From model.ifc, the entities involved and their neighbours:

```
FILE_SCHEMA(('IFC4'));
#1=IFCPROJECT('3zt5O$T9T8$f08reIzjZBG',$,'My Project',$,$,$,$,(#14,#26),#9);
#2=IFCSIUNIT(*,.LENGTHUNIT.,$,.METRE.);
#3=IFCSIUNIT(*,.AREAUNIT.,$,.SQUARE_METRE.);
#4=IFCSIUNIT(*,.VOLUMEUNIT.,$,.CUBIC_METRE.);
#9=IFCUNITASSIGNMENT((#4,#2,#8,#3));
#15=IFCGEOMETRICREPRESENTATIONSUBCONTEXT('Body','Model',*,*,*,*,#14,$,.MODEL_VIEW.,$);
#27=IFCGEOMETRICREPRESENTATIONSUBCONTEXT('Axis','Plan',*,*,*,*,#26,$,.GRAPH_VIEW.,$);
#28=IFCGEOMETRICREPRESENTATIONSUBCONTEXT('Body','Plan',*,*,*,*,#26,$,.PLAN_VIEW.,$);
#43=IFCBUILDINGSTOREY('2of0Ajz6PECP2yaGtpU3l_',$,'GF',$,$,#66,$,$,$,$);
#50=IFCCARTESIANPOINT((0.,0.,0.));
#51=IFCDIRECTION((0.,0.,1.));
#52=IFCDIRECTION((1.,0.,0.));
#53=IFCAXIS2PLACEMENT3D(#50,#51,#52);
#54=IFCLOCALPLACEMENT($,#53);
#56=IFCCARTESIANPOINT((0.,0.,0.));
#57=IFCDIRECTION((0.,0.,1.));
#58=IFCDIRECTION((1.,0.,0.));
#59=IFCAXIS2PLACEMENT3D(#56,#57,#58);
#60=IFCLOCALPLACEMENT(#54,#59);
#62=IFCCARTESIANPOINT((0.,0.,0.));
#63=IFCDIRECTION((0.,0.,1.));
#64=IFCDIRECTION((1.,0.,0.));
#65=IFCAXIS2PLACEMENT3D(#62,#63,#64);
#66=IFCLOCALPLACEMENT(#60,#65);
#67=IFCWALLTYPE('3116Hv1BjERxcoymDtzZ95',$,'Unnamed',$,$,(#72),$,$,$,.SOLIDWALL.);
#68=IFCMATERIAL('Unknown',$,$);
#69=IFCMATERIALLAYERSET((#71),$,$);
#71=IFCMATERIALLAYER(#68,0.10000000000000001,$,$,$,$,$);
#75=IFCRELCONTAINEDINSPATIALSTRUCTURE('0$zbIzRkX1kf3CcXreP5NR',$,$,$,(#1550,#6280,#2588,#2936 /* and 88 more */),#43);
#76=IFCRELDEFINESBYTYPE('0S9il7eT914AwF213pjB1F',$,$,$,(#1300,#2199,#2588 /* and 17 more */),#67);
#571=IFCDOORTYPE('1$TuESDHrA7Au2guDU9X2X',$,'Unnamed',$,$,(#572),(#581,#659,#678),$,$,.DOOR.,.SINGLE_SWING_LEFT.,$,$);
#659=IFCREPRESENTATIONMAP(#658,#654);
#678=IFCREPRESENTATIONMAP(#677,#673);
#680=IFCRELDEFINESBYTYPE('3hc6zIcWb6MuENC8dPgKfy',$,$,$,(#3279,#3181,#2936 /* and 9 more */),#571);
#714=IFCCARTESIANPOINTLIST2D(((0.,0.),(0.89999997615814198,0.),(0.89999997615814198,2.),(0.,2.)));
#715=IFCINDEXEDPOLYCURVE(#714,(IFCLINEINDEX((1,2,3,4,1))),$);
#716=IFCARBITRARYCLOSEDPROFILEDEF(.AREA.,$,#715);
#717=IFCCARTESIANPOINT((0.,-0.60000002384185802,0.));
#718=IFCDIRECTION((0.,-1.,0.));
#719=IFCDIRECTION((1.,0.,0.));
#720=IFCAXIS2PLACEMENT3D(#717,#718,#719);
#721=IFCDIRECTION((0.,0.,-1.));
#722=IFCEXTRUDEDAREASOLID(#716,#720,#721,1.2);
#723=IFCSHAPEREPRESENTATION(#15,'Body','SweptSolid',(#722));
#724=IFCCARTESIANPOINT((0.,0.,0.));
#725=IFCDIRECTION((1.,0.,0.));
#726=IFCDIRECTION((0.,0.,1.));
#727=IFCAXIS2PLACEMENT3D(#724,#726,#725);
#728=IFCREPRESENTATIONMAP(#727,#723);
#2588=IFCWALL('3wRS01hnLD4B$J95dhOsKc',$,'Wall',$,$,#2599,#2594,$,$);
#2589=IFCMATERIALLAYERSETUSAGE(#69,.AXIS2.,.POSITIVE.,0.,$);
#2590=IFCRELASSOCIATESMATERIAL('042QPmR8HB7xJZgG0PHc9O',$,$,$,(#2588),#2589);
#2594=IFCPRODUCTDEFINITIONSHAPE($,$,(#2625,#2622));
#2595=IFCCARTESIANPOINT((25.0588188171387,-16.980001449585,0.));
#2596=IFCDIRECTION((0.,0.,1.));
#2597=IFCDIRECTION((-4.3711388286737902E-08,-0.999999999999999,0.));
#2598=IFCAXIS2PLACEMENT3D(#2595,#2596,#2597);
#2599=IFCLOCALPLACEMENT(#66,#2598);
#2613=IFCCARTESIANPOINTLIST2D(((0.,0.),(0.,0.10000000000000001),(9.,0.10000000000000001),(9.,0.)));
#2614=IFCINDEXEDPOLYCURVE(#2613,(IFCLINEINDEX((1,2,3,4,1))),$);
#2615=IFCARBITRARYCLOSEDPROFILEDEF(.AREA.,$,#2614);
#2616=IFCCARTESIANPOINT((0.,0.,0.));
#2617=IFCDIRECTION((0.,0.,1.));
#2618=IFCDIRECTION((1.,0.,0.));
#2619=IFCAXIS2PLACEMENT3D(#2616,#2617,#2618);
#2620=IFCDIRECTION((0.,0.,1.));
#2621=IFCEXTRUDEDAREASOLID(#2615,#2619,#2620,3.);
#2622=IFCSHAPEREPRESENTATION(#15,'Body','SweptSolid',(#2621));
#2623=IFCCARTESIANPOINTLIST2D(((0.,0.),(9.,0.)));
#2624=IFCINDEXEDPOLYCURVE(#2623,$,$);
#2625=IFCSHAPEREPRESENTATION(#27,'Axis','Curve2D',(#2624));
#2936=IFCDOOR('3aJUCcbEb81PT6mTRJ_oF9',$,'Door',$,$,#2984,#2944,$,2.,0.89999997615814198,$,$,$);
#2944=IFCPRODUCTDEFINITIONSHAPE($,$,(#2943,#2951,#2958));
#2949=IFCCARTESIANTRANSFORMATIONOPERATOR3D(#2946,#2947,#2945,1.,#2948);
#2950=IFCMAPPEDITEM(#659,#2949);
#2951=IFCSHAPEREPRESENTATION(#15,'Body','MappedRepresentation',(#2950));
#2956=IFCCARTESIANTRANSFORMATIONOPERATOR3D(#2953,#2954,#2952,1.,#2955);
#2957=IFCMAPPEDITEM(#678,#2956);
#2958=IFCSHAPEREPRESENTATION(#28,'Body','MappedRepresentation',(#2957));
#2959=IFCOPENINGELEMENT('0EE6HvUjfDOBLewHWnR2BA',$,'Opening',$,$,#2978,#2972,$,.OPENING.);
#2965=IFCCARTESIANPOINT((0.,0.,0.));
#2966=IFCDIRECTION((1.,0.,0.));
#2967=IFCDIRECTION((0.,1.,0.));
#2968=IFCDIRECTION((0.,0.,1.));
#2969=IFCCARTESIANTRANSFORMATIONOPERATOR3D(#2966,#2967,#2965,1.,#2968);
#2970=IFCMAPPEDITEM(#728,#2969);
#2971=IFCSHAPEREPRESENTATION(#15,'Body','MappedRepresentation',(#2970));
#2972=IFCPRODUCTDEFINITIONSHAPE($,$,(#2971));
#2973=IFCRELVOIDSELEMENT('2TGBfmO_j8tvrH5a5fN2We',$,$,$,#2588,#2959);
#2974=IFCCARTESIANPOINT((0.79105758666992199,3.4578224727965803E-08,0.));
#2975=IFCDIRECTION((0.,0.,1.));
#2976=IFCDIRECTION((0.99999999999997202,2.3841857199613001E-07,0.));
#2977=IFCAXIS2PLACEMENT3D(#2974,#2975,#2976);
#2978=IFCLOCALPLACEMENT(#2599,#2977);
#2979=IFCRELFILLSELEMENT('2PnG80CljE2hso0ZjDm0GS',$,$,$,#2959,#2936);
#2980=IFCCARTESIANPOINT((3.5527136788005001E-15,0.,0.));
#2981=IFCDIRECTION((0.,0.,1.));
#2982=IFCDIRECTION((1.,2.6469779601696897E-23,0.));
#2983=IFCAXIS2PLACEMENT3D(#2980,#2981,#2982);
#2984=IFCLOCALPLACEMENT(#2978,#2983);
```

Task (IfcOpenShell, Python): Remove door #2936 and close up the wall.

```python
import ifcopenshell
import ifcopenshell.api.feature
import ifcopenshell.api.root
import ifcopenshell.geom
import ifcopenshell.util.shape

model = ifcopenshell.open("model.ifc")
settings = ifcopenshell.geom.settings()


def volume(element):
    """Net volume in cubic metres, openings subtracted."""
    shape = ifcopenshell.geom.create_shape(settings, element)
    return ifcopenshell.util.shape.get_volume(shape.geometry)


door = model.by_guid("3aJUCcbEb81PT6mTRJ_oF9")
opening = door.FillsVoids[0].RelatingOpeningElement
wall = opening.VoidsElements[0].RelatingBuildingElement
before = volume(wall)

ifcopenshell.api.root.remove_product(model, product=door)
ifcopenshell.api.feature.remove_feature(model, feature=opening)

after = volume(wall)

print(f"wall volume {before:.3f} -> {after:.3f} m3")

model.write("model_edited.ifc")
```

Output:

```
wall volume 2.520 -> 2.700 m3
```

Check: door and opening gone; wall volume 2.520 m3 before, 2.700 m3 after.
